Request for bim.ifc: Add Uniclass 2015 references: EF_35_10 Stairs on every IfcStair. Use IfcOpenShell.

First a look at what the model holds.

```python
import ifcopenshell

model = ifcopenshell.open("bim.ifc")
print(model.schema)
print("classifications:", [c.Name for c in model.by_type("IfcClassification")])
for ifc_class in ("IfcDoor", "IfcRoof", "IfcStair", "IfcWall", "IfcWindow"):
    print(ifc_class, len(model.by_type(ifc_class)))
```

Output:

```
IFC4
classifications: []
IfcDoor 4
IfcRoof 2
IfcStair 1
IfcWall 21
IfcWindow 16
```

```python
import ifcopenshell
import ifcopenshell.api.classification

model = ifcopenshell.open("bim.ifc")

system = ifcopenshell.api.classification.add_classification(model, classification="Uniclass 2015")

codes = {
    "IfcStair": ("EF_35_10", "Stairs"),
}
for ifc_class, (code, name) in codes.items():
    products = model.by_type(ifc_class)
    ifcopenshell.api.classification.add_reference(
        model, products=products, classification=system, identification=code, name=name
    )
    print(code, len(products))

model.write("bim_v2.ifc")
```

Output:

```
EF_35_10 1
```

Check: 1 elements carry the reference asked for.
